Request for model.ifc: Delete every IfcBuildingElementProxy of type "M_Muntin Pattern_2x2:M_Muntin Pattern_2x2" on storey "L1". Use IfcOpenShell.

First a look at what the model holds.

```python
import ifcopenshell
import ifcopenshell.util.element

model = ifcopenshell.open("model.ifc")
print(model.schema)
storey = next(s for s in model.by_type("IfcBuildingStorey") if s.Name == "L1")
proxies = [e for e in ifcopenshell.util.element.get_decomposition(storey) if e.is_a("IfcBuildingElementProxy")]
seen = {}
for e in proxies:
    element_type = ifcopenshell.util.element.get_type(e)
    name = element_type.Name if element_type not in (None, e) else None
    seen[name] = seen.get(name, 0) + 1
for name, count in sorted(seen.items(), key=str):
    print(count, "x", name)
```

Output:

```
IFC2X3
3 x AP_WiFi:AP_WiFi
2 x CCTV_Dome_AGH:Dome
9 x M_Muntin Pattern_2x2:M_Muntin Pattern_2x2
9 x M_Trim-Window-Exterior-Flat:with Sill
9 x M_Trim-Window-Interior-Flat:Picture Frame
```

```python
import ifcopenshell
import ifcopenshell.api.root
import ifcopenshell.util.element

model = ifcopenshell.open("model.ifc")

storey = next(s for s in model.by_type("IfcBuildingStorey") if s.Name == "L1")
proxies = [e for e in ifcopenshell.util.element.get_decomposition(storey) if e.is_a("IfcBuildingElementProxy")]
targets = [e for e in proxies if (t := ifcopenshell.util.element.get_type(e)) not in (None, e) and t.Name == "M_Muntin Pattern_2x2:M_Muntin Pattern_2x2"]

for e in targets:
    ifcopenshell.api.root.remove_product(model, product=e)
print(len(targets), "removed")

model.write("model_updated.ifc")
```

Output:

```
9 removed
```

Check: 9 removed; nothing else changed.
